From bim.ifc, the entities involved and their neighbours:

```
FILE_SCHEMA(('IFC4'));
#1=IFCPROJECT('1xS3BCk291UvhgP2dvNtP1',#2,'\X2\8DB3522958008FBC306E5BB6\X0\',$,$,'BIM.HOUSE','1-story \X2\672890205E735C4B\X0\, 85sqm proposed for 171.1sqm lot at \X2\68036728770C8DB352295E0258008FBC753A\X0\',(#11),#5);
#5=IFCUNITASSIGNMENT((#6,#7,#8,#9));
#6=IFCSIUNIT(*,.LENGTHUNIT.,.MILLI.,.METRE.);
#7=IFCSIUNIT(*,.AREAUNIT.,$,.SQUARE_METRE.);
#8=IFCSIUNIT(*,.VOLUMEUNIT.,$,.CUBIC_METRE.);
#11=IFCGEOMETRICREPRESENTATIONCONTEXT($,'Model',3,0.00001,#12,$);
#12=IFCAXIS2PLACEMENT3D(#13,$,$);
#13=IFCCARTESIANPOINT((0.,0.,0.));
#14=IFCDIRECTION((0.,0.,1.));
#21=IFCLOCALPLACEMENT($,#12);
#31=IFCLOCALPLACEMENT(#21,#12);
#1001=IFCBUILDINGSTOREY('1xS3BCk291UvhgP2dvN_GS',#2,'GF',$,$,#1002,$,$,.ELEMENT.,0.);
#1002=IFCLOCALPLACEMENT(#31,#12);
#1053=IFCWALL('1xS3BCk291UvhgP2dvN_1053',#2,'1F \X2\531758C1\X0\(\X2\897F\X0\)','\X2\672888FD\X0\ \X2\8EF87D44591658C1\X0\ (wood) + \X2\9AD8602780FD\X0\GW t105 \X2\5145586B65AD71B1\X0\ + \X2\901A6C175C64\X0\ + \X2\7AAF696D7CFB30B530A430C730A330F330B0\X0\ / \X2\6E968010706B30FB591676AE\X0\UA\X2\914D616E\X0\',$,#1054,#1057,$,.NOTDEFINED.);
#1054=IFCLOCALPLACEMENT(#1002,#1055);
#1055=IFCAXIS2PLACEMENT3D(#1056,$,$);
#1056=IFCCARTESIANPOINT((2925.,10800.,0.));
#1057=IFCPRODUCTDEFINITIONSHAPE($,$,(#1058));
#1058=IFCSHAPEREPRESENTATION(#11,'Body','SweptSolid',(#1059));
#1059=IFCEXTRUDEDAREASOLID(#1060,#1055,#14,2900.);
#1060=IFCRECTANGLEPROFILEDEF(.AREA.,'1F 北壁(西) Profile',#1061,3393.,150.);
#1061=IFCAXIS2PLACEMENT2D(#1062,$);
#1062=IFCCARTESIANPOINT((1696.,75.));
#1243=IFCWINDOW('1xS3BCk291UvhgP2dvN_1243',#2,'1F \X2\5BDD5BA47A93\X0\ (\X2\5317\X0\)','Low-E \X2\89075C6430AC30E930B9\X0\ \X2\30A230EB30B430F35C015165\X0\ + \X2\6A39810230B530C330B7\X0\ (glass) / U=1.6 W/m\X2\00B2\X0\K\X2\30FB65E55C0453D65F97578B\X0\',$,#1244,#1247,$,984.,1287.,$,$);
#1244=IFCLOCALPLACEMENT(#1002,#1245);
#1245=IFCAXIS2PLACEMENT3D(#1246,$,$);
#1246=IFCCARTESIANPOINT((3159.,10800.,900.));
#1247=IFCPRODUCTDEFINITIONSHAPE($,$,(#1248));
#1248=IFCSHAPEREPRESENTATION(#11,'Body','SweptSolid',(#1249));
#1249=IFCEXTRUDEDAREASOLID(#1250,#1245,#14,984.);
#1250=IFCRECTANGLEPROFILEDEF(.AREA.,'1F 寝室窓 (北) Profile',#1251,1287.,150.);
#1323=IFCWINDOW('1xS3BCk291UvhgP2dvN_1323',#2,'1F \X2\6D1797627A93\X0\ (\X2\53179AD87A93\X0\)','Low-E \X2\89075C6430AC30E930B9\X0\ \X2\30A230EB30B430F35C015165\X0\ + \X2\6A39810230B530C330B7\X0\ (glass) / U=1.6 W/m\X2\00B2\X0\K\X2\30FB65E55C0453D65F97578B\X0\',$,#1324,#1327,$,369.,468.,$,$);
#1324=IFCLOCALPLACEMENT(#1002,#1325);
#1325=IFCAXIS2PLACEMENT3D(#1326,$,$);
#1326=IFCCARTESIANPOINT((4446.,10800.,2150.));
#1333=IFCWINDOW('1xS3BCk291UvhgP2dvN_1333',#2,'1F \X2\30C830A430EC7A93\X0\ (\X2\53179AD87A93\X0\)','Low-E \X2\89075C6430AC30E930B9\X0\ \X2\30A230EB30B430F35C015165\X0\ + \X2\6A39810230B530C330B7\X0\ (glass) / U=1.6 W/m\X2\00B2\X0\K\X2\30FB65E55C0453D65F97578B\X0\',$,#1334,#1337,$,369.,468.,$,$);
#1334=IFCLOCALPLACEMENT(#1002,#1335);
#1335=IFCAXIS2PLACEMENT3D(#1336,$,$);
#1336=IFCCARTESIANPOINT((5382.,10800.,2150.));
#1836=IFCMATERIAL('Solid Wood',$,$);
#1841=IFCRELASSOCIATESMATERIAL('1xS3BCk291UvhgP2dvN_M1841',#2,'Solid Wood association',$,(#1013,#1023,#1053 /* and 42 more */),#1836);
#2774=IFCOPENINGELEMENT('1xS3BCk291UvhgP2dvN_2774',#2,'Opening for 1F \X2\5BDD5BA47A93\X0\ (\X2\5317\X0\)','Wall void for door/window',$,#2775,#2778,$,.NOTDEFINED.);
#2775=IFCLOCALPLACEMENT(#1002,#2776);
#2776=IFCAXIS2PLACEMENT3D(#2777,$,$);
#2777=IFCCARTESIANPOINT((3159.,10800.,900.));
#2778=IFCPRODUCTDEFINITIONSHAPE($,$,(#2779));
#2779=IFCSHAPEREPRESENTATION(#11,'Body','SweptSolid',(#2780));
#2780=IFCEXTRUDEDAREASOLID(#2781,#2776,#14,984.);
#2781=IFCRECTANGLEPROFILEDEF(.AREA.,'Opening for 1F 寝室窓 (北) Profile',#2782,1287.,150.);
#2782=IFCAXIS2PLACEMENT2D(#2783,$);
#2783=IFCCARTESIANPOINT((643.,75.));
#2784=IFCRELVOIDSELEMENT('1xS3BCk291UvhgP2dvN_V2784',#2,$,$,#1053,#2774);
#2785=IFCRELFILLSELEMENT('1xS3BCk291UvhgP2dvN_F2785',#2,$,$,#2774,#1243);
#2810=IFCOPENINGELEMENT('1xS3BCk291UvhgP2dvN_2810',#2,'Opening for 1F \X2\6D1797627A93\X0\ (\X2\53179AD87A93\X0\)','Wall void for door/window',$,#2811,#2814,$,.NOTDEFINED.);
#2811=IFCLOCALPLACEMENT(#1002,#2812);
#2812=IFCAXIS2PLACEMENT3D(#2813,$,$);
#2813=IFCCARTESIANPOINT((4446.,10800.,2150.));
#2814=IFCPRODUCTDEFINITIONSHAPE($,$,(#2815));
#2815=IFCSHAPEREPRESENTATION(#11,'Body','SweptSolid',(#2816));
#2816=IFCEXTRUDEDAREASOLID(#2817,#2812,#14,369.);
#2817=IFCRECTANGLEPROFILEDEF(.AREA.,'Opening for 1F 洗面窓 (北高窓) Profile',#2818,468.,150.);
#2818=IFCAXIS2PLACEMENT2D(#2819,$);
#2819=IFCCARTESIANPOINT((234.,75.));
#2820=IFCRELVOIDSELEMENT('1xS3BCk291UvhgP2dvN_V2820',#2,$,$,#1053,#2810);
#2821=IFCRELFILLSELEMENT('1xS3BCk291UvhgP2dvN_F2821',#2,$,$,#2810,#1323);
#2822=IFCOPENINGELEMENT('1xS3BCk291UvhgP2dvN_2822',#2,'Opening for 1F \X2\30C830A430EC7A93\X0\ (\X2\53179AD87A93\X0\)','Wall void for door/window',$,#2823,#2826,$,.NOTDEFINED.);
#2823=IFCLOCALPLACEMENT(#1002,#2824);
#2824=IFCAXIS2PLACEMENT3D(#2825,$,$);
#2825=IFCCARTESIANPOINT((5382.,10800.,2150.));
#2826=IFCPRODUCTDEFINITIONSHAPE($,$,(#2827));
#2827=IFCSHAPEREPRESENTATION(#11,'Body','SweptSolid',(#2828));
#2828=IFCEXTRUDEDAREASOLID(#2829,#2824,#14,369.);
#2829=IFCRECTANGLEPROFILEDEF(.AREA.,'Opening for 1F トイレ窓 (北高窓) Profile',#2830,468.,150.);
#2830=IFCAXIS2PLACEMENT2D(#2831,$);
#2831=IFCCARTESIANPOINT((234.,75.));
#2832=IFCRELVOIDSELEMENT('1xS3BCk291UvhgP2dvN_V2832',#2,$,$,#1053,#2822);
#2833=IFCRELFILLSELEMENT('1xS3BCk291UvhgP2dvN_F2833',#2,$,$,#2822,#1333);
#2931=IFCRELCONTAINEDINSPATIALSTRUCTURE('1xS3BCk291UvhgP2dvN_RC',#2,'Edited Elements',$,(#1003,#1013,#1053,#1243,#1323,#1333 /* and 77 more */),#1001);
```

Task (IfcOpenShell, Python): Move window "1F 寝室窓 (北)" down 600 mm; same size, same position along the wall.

```python
import numpy as np
import ifcopenshell
import ifcopenshell.api.geometry
import ifcopenshell.util.placement
import ifcopenshell.util.unit

model = ifcopenshell.open("bim.ifc")
unit_scale = ifcopenshell.util.unit.calculate_unit_scale(model)

window = model.by_guid("1xS3BCk291UvhgP2dvN_1243")
opening = window.FillsVoids[0].RelatingOpeningElement
dz = -0.6 / unit_scale

shift = np.array([0.0, 0.0, dz])
# The window is not placed relative to its opening, so move both.
for product in (opening, window):
    matrix = ifcopenshell.util.placement.get_local_placement(product.ObjectPlacement)
    matrix[:3, 3] += shift
    ifcopenshell.api.geometry.edit_object_placement(model, product=product, matrix=matrix, is_si=False)

print(f"moved by {dz * unit_scale:+.3f} m")

model.write("bim_updated.ifc")
```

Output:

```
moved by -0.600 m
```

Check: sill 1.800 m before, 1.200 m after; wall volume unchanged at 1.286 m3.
